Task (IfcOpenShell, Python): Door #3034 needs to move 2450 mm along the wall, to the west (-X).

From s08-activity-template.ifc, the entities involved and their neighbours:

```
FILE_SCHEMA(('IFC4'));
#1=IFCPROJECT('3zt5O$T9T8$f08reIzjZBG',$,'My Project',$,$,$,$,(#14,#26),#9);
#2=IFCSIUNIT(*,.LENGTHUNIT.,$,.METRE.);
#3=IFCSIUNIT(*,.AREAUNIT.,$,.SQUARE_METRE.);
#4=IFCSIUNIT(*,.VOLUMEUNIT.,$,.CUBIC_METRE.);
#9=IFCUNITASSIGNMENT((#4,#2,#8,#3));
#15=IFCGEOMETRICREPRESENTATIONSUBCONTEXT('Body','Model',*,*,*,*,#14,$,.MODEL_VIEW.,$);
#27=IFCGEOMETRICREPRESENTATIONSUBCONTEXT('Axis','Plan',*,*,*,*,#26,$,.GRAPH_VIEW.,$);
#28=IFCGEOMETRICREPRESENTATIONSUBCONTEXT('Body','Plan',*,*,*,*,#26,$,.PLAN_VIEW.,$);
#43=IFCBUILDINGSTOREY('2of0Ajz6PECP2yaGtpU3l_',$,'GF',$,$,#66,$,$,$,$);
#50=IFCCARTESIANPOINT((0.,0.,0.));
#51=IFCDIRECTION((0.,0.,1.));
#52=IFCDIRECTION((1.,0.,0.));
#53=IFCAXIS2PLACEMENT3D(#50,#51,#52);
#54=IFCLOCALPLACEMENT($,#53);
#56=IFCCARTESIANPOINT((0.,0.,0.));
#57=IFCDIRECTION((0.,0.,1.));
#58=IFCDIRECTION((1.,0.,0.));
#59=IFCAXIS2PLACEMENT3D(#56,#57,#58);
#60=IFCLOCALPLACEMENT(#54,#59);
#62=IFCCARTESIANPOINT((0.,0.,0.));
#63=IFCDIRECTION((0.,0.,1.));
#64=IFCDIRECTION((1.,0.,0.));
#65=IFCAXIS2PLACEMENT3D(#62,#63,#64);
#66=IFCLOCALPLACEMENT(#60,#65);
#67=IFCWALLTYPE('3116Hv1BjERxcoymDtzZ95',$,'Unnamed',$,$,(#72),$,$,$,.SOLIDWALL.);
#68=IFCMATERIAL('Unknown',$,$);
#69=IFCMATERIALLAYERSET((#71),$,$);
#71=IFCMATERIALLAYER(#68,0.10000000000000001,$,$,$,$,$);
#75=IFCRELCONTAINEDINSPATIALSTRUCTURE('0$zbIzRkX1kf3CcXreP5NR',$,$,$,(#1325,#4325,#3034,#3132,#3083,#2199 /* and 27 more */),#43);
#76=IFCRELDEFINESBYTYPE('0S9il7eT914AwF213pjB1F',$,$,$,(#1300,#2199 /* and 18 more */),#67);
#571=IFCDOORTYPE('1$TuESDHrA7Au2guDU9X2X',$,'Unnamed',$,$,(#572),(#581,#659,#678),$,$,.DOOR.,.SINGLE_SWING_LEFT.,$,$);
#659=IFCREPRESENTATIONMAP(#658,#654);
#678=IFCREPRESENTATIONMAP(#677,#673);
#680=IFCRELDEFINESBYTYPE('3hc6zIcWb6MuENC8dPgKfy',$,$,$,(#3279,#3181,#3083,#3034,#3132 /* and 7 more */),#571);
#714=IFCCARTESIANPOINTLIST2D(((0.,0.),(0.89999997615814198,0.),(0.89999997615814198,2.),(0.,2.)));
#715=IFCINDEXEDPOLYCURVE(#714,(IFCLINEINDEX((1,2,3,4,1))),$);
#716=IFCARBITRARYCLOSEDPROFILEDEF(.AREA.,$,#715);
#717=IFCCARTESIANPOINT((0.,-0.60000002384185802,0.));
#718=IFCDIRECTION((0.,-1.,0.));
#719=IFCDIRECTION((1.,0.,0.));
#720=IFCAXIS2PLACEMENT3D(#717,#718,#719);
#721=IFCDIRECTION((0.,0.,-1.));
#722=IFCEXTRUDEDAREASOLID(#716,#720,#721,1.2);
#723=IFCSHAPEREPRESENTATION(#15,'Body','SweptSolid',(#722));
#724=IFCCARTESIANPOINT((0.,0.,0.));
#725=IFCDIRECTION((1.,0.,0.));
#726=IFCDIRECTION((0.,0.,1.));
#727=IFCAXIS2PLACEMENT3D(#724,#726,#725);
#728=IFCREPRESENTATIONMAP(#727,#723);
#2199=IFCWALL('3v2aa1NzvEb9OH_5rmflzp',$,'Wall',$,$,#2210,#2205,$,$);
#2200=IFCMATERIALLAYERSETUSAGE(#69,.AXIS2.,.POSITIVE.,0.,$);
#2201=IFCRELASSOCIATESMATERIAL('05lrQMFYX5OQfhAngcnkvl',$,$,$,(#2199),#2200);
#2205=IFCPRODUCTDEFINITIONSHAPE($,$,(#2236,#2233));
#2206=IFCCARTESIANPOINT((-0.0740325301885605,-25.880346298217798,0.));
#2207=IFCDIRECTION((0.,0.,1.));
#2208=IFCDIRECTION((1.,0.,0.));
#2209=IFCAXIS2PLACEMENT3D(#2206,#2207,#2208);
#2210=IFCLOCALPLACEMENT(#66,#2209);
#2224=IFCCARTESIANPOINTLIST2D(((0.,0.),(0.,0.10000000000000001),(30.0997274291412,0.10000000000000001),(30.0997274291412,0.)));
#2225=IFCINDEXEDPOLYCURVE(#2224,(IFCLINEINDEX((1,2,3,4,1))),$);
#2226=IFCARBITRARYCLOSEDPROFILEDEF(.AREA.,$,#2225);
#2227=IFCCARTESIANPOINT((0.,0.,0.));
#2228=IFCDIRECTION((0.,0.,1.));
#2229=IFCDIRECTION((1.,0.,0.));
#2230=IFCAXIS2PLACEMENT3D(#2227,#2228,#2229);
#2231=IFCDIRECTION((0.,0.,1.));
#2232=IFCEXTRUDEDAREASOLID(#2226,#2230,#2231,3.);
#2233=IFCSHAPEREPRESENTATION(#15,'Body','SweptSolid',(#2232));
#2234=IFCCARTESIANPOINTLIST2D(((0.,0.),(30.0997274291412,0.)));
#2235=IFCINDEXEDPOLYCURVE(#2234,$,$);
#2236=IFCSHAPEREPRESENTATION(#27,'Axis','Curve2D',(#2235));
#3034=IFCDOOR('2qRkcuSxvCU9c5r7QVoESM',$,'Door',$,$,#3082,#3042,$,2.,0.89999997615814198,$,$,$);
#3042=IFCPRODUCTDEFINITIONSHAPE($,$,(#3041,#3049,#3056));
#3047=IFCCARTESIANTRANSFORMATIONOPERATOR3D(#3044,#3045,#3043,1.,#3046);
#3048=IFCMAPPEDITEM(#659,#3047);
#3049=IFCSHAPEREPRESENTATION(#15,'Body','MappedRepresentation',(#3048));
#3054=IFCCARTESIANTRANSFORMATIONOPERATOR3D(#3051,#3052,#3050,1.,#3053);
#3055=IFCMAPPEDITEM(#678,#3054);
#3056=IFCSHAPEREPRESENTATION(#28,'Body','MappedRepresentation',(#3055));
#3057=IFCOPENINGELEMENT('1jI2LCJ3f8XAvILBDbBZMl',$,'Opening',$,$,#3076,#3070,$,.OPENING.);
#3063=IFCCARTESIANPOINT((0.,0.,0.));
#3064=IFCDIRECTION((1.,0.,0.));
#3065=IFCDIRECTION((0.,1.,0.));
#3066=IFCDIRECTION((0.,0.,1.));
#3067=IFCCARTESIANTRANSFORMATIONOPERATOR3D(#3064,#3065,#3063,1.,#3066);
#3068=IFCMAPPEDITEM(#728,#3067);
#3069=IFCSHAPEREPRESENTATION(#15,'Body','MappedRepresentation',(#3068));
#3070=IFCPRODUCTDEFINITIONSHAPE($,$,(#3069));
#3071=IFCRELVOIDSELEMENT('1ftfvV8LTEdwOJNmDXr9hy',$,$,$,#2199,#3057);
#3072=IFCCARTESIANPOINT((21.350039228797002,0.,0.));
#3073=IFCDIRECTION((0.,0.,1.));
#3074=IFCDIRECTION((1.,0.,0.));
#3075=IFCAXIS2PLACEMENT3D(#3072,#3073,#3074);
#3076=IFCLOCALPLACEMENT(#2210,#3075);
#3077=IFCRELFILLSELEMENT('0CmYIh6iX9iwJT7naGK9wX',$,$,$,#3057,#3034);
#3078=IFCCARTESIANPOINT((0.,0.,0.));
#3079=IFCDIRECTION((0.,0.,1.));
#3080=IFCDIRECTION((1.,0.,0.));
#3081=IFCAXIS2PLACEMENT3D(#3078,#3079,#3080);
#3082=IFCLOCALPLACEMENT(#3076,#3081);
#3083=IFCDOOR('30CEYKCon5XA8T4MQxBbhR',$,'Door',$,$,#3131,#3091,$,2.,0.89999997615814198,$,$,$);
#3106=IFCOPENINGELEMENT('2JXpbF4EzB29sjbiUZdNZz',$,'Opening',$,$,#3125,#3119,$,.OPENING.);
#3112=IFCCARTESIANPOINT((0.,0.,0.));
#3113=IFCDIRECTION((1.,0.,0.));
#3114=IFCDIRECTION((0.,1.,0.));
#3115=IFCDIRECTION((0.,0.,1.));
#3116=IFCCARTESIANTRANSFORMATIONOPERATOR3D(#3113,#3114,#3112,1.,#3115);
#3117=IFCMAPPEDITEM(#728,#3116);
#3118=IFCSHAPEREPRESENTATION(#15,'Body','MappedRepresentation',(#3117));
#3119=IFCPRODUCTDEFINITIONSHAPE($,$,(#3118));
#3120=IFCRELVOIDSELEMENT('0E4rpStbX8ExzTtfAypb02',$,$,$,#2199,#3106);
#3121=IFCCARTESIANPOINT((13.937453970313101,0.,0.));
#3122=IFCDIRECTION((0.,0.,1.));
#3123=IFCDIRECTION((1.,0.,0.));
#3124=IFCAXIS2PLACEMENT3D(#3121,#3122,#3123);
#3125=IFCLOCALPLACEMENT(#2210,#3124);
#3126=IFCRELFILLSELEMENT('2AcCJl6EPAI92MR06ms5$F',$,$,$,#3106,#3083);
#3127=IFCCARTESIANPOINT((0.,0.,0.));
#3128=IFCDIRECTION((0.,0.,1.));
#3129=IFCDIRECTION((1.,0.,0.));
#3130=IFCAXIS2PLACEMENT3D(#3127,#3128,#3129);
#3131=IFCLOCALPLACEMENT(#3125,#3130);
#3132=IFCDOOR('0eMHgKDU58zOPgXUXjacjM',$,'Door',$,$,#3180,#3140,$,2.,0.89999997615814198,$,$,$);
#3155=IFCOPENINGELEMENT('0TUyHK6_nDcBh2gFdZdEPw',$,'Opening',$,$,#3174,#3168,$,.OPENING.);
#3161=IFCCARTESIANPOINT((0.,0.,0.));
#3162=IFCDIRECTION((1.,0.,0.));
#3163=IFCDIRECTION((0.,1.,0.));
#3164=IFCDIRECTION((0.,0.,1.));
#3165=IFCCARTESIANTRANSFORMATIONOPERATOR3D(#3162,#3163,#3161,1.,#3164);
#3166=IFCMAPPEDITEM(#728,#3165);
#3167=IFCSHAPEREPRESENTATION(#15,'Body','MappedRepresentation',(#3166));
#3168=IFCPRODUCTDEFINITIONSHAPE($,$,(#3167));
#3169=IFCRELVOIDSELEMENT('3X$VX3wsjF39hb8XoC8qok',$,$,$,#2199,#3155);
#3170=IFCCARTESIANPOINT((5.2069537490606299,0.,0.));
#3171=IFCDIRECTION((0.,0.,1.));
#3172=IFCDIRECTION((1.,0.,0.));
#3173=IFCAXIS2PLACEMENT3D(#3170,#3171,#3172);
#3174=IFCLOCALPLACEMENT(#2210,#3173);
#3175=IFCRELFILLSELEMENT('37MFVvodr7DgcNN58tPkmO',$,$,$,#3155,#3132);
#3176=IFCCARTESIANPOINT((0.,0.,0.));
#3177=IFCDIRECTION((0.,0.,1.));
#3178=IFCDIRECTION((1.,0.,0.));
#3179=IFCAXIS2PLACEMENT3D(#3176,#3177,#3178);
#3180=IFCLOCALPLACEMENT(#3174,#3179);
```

```python
import ifcopenshell
import ifcopenshell.api.geometry
import ifcopenshell.util.placement
import ifcopenshell.util.unit

model = ifcopenshell.open("s08-activity-template.ifc")
unit_scale = ifcopenshell.util.unit.calculate_unit_scale(model)

door = model.by_id(3034)
opening = door.FillsVoids[0].RelatingOpeningElement
wall = opening.VoidsElements[0].RelatingBuildingElement

wall_matrix = ifcopenshell.util.placement.get_local_placement(wall.ObjectPlacement)
shift = wall_matrix[:3, 0] * -2.45 / unit_scale
before = ifcopenshell.util.placement.get_local_placement(door.ObjectPlacement)[:3, 3].copy()

# The door is placed relative to its opening, so it follows when the opening moves.
matrix = ifcopenshell.util.placement.get_local_placement(opening.ObjectPlacement)
matrix[:3, 3] += shift
ifcopenshell.api.geometry.edit_object_placement(
    model, product=opening, matrix=matrix, is_si=False, should_transform_children=True
)

after = ifcopenshell.util.placement.get_local_placement(door.ObjectPlacement)[:3, 3]
print("door moved by", (after - before).round(3) + 0.0)

model.write("s08-activity-template-out.ifc")
```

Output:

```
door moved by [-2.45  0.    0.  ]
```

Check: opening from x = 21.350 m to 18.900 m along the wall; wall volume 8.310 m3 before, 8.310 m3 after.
